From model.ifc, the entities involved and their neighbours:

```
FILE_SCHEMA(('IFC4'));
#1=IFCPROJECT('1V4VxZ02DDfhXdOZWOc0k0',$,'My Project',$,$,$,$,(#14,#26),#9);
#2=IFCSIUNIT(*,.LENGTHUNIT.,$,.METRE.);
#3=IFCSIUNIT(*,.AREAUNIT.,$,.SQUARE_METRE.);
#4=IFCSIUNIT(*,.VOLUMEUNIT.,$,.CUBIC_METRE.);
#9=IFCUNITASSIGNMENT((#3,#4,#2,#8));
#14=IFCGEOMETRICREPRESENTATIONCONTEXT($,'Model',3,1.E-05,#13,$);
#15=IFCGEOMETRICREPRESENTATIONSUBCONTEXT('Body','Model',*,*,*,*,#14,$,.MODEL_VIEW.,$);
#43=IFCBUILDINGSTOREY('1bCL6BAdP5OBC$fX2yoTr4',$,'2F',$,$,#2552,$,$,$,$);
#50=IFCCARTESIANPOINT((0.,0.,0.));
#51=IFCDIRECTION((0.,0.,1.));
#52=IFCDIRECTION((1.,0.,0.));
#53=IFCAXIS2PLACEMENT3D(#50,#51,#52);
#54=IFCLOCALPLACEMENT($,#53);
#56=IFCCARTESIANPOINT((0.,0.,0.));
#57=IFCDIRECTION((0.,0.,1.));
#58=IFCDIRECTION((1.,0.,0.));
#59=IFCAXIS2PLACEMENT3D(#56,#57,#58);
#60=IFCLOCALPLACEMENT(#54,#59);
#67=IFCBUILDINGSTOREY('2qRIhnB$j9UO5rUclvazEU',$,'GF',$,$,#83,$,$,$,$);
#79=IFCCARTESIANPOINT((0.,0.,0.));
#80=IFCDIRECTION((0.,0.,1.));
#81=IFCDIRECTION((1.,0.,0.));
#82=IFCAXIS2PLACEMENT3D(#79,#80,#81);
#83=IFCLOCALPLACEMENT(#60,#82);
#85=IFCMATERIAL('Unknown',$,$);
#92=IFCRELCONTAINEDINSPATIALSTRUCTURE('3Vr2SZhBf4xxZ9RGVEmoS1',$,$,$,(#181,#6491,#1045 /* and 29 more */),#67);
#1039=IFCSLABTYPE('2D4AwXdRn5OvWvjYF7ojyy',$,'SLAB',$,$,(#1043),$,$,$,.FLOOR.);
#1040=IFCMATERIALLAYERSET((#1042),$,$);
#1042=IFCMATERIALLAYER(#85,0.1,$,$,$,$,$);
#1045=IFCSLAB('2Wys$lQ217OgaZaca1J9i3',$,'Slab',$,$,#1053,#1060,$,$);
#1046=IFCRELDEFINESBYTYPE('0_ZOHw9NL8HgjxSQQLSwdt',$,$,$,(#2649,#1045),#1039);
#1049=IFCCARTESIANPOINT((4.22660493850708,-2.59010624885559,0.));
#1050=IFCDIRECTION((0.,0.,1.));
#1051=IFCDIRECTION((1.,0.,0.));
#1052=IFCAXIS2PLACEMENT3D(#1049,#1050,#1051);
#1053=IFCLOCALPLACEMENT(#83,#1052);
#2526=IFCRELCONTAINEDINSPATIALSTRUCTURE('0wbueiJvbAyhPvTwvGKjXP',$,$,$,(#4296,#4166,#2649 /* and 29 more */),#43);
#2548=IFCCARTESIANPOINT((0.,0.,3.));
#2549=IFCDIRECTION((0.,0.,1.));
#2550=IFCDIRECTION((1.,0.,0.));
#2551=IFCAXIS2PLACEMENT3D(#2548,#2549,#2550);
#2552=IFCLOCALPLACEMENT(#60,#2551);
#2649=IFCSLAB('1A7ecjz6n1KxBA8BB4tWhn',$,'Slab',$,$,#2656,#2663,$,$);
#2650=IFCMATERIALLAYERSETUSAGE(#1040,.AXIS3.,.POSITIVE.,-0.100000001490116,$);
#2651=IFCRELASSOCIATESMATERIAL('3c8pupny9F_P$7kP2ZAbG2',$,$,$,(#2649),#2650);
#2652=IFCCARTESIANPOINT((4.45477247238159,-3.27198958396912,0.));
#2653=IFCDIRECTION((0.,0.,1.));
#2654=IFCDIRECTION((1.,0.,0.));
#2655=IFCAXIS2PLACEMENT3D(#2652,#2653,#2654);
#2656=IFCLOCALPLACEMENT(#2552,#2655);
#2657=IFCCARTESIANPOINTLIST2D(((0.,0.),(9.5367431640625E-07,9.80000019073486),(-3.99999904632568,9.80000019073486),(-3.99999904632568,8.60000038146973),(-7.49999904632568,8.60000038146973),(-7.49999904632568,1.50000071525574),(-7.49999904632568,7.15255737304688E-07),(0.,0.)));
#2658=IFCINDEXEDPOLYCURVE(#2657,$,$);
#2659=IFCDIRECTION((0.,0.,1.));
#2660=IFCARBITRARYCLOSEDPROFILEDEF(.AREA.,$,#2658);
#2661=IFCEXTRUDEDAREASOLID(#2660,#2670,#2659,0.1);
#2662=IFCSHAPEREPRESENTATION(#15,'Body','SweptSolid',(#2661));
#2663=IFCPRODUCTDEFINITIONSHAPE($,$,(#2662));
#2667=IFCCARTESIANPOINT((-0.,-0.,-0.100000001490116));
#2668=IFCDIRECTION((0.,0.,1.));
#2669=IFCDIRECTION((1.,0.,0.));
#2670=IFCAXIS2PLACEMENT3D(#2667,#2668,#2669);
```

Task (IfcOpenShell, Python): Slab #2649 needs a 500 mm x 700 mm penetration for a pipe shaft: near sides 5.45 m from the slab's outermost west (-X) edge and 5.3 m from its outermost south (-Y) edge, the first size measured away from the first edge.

```python
import numpy as np
import ifcopenshell
import ifcopenshell.api.feature
import ifcopenshell.api.geometry
import ifcopenshell.api.root
import ifcopenshell.geom
import ifcopenshell.util.placement
import ifcopenshell.util.representation
import ifcopenshell.util.shape
import ifcopenshell.util.unit

model = ifcopenshell.open("model.ifc")
unit_scale = ifcopenshell.util.unit.calculate_unit_scale(model)
settings = ifcopenshell.geom.settings()


def volume(element):
    """Net volume in cubic metres, openings subtracted."""
    shape = ifcopenshell.geom.create_shape(settings, element)
    return ifcopenshell.util.shape.get_volume(shape.geometry)


slab = model.by_guid("1A7ecjz6n1KxBA8BB4tWhn")
before = volume(slab)

# Extent in the slab's own axes, in metres. The edges named are its -X and -Y sides.
slab_shape = ifcopenshell.geom.create_shape(settings, slab)
vertices = ifcopenshell.util.shape.get_vertices(slab_shape.geometry)
x_min, y_min, bottom = vertices.min(axis=0)
top = vertices[:, 2].max()

opening = ifcopenshell.api.root.create_entity(model, ifc_class="IfcOpeningElement", name="Pipe shaft opening", predefined_type="OPENING")
context = ifcopenshell.util.representation.get_context(model, "Model", "Body", "MODEL_VIEW")
width, depth = 0.5, 0.7
outline = [(0.0, 0.0), (width, 0.0), (width, depth), (0.0, depth), (0.0, 0.0)]
# Overshoot both faces by 50 mm so the cut is clean.
shape = ifcopenshell.api.geometry.add_slab_representation(
    model, context=context, depth=top - bottom + 0.1, polyline=outline
)
ifcopenshell.api.geometry.assign_representation(model, product=opening, representation=shape)

matrix = ifcopenshell.util.placement.get_local_placement(slab.ObjectPlacement)
matrix[:, 3] = matrix @ np.append(np.array([x_min + 5.45, y_min + 5.3, bottom - 0.05]) / unit_scale, 1.0)
ifcopenshell.api.geometry.edit_object_placement(model, product=opening, matrix=matrix, is_si=False)
ifcopenshell.api.feature.add_feature(model, feature=opening, element=slab)

after = volume(slab)

print(f"slab volume {before:.3f} -> {after:.3f} m3")

model.write("model_edited.ifc")
```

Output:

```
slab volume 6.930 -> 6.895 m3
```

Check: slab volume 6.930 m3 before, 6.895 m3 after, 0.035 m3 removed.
